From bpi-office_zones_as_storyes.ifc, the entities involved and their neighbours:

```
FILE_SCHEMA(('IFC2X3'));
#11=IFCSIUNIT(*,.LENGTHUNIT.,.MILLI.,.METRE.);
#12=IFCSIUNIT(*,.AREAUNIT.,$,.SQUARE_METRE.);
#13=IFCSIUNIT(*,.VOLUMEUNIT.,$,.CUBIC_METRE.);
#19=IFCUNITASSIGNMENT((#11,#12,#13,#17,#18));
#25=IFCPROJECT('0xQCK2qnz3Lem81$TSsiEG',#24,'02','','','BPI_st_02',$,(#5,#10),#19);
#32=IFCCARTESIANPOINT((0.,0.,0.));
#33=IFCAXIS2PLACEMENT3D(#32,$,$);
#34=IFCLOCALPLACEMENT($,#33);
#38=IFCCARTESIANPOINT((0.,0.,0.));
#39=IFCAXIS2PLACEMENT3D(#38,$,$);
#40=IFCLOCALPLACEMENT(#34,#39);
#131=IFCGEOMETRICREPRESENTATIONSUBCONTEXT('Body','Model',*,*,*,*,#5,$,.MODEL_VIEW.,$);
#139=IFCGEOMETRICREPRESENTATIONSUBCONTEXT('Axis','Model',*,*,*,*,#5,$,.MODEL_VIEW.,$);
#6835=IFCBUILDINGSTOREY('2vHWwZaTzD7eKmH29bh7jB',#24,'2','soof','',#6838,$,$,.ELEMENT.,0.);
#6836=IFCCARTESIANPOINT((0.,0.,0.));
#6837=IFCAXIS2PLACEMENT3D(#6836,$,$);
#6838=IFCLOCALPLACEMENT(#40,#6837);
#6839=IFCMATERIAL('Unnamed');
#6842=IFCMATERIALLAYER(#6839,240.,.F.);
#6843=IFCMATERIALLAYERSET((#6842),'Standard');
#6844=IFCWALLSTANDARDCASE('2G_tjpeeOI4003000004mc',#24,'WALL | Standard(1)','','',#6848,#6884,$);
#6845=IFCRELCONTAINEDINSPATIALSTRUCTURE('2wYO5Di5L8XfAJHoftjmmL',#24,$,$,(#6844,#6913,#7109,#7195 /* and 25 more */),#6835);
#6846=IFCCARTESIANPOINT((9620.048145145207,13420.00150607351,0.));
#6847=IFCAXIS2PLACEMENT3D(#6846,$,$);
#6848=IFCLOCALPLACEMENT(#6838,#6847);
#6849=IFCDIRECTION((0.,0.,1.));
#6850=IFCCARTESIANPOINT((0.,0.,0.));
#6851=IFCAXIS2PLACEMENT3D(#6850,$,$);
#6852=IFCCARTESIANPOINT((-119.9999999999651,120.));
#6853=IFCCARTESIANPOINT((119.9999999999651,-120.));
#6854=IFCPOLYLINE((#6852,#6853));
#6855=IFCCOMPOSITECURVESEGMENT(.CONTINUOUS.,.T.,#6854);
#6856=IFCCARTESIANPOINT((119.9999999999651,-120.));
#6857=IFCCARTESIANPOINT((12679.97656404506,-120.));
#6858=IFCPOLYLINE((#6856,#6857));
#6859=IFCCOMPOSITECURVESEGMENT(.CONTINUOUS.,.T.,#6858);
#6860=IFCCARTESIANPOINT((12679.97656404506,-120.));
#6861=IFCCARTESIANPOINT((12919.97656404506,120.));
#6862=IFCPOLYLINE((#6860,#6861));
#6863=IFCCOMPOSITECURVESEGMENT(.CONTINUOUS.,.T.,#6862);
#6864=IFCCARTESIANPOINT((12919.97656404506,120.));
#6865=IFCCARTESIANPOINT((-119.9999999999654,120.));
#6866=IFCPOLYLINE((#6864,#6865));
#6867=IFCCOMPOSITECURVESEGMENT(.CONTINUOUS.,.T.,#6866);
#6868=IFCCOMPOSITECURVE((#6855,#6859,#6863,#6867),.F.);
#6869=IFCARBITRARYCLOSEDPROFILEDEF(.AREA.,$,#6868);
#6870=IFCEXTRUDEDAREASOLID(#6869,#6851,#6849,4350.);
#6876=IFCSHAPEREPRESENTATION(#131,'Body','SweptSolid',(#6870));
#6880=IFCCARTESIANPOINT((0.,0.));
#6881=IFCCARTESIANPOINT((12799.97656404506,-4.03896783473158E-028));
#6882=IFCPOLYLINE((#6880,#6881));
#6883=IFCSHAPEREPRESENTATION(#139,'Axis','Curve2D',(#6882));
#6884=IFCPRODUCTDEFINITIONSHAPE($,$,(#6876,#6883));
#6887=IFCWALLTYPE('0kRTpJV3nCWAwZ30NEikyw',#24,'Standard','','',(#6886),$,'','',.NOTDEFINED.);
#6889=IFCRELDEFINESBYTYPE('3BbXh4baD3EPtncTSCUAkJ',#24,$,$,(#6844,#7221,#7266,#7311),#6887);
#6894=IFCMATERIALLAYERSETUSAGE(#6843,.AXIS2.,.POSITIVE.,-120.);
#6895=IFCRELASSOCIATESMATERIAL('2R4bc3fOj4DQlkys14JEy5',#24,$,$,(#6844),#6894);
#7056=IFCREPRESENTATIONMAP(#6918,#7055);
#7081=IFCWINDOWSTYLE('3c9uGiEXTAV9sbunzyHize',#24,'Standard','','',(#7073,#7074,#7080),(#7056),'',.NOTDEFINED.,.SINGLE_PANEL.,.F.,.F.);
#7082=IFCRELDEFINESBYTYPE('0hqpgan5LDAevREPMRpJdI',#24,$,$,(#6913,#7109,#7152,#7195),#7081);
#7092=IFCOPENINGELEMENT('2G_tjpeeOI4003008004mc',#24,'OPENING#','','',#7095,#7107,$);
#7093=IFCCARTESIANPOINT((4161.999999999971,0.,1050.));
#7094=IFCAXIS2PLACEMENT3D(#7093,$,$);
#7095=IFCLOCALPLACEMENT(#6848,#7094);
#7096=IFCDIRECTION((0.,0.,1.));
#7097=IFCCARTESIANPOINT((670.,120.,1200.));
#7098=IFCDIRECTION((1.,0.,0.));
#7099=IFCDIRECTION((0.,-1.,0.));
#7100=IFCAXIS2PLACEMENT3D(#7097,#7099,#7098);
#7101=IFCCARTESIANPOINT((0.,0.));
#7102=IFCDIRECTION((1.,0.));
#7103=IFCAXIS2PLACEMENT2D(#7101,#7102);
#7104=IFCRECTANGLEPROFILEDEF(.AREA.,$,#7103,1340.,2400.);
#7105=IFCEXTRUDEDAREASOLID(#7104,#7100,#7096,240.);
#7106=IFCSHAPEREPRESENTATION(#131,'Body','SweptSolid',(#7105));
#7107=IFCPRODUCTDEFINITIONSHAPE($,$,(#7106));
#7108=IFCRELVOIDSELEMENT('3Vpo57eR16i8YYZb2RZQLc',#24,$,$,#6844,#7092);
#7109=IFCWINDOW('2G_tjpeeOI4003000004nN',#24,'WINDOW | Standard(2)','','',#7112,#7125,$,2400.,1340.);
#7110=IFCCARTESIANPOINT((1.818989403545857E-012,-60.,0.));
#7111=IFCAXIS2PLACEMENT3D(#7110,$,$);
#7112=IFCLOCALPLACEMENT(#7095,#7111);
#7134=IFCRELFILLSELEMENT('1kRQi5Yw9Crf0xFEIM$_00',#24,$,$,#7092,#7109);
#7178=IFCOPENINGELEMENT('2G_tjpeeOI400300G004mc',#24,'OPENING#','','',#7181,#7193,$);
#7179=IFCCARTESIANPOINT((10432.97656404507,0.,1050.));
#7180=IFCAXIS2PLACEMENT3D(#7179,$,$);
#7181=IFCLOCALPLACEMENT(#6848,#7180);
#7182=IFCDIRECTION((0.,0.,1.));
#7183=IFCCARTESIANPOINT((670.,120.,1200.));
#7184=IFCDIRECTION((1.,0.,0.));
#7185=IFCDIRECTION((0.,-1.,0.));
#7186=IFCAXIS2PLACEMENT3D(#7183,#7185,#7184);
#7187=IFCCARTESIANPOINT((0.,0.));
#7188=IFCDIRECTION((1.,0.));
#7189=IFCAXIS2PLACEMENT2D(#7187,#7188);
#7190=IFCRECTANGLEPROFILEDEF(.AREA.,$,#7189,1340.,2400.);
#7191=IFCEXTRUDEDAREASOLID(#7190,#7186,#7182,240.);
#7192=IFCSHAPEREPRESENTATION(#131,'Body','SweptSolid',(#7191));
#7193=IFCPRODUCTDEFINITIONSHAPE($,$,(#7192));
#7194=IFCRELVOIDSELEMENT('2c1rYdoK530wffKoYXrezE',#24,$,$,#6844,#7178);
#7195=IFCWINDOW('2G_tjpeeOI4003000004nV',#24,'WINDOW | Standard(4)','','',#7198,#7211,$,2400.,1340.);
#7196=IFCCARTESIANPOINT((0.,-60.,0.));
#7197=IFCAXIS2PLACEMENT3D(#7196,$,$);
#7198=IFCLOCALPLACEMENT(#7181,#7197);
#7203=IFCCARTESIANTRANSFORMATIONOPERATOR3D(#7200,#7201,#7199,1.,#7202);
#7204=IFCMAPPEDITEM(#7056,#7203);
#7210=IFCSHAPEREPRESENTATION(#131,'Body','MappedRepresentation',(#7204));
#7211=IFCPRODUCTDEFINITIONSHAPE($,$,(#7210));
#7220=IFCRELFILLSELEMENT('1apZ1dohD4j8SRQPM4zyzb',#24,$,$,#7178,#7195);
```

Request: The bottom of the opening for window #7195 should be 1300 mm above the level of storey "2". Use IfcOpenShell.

```python
import numpy as np
import ifcopenshell
import ifcopenshell.api.geometry
import ifcopenshell.geom
import ifcopenshell.util.element
import ifcopenshell.util.placement
import ifcopenshell.util.shape
import ifcopenshell.util.unit

model = ifcopenshell.open("bpi-office_zones_as_storyes.ifc")
unit_scale = ifcopenshell.util.unit.calculate_unit_scale(model)

window = model.by_guid("2G_tjpeeOI4003000004nV")
opening = window.FillsVoids[0].RelatingOpeningElement
storey = ifcopenshell.util.element.get_container(window, ifc_class="IfcBuildingStorey")
level = ifcopenshell.util.placement.get_local_placement(storey.ObjectPlacement)[2, 3]

# The opening's origin need not be at the sill, so measure its lowest point.
shape = ifcopenshell.geom.create_shape(ifcopenshell.geom.settings(), opening)
bottom = ifcopenshell.util.shape.get_shape_bottom_elevation(shape, shape.geometry) / unit_scale
dz = level + 1.3 / unit_scale - bottom

shift = np.array([0.0, 0.0, dz])
# The window is placed relative to its opening, so it follows when the opening moves.
matrix = ifcopenshell.util.placement.get_local_placement(opening.ObjectPlacement)
matrix[:3, 3] += shift
ifcopenshell.api.geometry.edit_object_placement(
    model, product=opening, matrix=matrix, is_si=False, should_transform_children=True
)

print(f"moved by {dz * unit_scale:+.3f} m")

model.write("bpi-office_zones_as_storyes_v2.ifc")
```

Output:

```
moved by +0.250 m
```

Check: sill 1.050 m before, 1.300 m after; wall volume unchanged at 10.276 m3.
